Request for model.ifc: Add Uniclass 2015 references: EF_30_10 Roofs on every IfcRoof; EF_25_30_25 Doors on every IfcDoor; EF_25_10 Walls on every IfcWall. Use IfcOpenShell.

First a look at what the model holds.

```python
import ifcopenshell

model = ifcopenshell.open("model.ifc")
print(model.schema)
print("classifications:", [c.Name for c in model.by_type("IfcClassification")])
for ifc_class in ("IfcDoor", "IfcRoof", "IfcStair", "IfcWall", "IfcWindow"):
    print(ifc_class, len(model.by_type(ifc_class)))
```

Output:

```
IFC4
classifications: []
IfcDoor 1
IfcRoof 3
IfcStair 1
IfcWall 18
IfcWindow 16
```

```python
import ifcopenshell
import ifcopenshell.api.classification

model = ifcopenshell.open("model.ifc")

system = ifcopenshell.api.classification.add_classification(model, classification="Uniclass 2015")

codes = {
    "IfcRoof": ("EF_30_10", "Roofs"),
    "IfcDoor": ("EF_25_30_25", "Doors"),
    "IfcWall": ("EF_25_10", "Walls"),
}
for ifc_class, (code, name) in codes.items():
    products = model.by_type(ifc_class)
    ifcopenshell.api.classification.add_reference(
        model, products=products, classification=system, identification=code, name=name
    )
    print(code, len(products))

model.write("model-out.ifc")
```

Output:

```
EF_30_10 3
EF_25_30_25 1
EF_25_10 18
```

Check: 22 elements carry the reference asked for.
